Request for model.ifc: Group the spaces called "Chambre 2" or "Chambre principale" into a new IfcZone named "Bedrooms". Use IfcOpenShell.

First a look at what the model holds.

```python
import ifcopenshell

model = ifcopenshell.open("model.ifc")
print(model.schema)
seen = {}
for space in model.by_type("IfcSpace"):
    seen[space.LongName] = seen.get(space.LongName, 0) + 1
for name, count in sorted(seen.items(), key=str):
    print(count, "x", name)
print("zones:", [z.Name for z in model.by_type("IfcZone")][:20])
```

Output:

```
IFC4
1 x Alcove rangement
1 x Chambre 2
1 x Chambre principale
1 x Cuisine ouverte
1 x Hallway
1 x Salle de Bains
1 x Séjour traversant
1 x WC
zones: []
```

```python
import ifcopenshell
import ifcopenshell.api.group
import ifcopenshell.api.root

model = ifcopenshell.open("model.ifc")

names = {"Chambre 2", "Chambre principale"}
spaces = [s for s in model.by_type("IfcSpace") if s.LongName in names]

zone = ifcopenshell.api.root.create_entity(model, ifc_class="IfcZone", name="Bedrooms")
ifcopenshell.api.group.assign_group(model, products=spaces, group=zone)
print(len(spaces), "spaces in", zone.Name)

model.write("model_v2.ifc")
```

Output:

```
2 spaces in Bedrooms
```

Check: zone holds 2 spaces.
